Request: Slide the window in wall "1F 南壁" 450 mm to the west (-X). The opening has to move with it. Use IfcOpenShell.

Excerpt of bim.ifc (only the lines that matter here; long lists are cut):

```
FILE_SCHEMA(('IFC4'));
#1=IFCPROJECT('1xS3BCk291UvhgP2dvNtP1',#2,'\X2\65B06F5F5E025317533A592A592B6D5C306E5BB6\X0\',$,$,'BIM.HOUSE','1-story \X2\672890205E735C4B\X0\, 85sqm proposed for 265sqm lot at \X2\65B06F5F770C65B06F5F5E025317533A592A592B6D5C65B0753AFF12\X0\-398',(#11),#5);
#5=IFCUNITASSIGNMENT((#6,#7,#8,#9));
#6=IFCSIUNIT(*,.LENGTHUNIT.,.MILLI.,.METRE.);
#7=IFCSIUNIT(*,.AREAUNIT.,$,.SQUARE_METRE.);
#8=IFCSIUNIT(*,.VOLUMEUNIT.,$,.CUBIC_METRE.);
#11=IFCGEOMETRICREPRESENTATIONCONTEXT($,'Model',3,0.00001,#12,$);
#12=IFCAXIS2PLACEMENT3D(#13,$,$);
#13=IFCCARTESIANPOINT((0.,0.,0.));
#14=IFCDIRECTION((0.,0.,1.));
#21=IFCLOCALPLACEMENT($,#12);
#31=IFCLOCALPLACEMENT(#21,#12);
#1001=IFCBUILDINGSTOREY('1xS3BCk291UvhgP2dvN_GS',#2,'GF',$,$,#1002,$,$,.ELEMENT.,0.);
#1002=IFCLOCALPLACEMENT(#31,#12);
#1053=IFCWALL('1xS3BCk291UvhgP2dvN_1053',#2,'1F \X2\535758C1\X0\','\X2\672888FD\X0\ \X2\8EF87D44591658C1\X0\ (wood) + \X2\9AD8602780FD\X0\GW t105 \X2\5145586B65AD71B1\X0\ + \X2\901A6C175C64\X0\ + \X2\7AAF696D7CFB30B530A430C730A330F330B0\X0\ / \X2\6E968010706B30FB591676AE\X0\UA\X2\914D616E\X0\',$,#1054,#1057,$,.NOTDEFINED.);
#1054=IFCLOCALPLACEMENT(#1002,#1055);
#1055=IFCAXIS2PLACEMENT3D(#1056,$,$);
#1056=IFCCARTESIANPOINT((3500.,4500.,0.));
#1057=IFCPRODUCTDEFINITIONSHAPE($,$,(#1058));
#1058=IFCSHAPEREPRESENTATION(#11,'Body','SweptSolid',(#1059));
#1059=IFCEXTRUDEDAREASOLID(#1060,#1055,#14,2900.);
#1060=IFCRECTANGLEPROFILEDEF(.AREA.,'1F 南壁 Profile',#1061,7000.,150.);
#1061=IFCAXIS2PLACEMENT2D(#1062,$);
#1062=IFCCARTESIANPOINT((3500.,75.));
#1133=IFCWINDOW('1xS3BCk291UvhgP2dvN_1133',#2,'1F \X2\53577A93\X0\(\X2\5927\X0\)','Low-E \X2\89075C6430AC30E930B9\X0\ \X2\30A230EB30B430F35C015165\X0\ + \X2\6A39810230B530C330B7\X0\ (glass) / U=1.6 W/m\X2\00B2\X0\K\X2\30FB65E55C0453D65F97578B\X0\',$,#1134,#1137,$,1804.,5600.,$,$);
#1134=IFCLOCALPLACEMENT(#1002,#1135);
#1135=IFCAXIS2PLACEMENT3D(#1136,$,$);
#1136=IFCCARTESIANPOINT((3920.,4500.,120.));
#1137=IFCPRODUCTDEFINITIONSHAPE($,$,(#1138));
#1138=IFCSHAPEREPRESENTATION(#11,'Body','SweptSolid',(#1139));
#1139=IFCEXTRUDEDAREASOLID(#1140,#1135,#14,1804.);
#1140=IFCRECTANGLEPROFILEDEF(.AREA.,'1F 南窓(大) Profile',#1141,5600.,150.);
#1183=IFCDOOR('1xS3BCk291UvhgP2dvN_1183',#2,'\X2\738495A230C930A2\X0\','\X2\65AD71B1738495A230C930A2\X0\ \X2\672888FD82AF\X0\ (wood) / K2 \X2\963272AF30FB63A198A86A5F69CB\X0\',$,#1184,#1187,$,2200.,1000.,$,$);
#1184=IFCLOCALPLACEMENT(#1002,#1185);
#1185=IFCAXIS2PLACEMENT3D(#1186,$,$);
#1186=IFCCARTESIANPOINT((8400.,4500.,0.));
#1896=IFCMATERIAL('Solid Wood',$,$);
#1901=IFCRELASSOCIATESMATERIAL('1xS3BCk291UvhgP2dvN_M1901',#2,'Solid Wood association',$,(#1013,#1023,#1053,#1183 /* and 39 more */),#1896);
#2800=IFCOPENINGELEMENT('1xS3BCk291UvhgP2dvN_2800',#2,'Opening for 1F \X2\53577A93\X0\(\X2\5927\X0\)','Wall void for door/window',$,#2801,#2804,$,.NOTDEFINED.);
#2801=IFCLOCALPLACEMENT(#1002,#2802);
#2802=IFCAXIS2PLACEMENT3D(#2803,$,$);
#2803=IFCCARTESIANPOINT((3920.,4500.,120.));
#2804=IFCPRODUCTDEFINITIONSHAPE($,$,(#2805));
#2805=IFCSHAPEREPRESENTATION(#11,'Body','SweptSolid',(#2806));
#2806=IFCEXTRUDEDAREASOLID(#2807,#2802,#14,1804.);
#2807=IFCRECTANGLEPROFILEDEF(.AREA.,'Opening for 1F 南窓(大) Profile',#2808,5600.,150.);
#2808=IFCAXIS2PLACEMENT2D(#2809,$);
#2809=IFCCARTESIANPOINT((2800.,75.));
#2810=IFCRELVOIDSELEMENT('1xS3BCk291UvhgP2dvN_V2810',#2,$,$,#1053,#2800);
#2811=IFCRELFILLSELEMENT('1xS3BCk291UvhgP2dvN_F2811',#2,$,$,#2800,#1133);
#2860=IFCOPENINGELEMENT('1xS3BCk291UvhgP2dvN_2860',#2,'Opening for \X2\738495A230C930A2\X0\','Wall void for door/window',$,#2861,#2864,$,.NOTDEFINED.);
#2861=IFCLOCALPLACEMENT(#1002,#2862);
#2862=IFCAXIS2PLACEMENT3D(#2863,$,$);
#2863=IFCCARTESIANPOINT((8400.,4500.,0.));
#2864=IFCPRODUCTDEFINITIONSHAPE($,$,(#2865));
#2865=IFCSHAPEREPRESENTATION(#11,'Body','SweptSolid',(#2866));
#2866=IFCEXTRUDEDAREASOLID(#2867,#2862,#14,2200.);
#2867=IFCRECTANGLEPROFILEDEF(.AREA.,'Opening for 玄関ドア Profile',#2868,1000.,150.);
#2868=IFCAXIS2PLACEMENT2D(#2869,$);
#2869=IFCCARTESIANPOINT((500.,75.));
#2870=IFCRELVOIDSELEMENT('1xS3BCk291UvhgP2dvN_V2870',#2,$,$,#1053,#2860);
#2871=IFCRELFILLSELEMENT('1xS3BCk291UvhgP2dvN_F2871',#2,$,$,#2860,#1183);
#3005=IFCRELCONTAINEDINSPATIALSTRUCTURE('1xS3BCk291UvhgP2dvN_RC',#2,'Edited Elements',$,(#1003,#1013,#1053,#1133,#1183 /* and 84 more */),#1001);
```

```python
import ifcopenshell
import ifcopenshell.api.geometry
import ifcopenshell.util.placement

model = ifcopenshell.open("bim.ifc")

window = model.by_guid("1xS3BCk291UvhgP2dvN_1133")
opening = window.FillsVoids[0].RelatingOpeningElement
wall = opening.VoidsElements[0].RelatingBuildingElement

wall_matrix = ifcopenshell.util.placement.get_local_placement(wall.ObjectPlacement)
shift = wall_matrix[:3, 0] * -450.0
before = ifcopenshell.util.placement.get_local_placement(window.ObjectPlacement)[:3, 3].copy()

# The window is not placed relative to its opening, so move both.
for product in (opening, window):
    matrix = ifcopenshell.util.placement.get_local_placement(product.ObjectPlacement)
    matrix[:3, 3] += shift
    ifcopenshell.api.geometry.edit_object_placement(model, product=product, matrix=matrix, is_si=False)

after = ifcopenshell.util.placement.get_local_placement(window.ObjectPlacement)[:3, 3]
print("window moved by", (after - before).round(3) + 0.0)

model.write("bim_updated.ifc")
```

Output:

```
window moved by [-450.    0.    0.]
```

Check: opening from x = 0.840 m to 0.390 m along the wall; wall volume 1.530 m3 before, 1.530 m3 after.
